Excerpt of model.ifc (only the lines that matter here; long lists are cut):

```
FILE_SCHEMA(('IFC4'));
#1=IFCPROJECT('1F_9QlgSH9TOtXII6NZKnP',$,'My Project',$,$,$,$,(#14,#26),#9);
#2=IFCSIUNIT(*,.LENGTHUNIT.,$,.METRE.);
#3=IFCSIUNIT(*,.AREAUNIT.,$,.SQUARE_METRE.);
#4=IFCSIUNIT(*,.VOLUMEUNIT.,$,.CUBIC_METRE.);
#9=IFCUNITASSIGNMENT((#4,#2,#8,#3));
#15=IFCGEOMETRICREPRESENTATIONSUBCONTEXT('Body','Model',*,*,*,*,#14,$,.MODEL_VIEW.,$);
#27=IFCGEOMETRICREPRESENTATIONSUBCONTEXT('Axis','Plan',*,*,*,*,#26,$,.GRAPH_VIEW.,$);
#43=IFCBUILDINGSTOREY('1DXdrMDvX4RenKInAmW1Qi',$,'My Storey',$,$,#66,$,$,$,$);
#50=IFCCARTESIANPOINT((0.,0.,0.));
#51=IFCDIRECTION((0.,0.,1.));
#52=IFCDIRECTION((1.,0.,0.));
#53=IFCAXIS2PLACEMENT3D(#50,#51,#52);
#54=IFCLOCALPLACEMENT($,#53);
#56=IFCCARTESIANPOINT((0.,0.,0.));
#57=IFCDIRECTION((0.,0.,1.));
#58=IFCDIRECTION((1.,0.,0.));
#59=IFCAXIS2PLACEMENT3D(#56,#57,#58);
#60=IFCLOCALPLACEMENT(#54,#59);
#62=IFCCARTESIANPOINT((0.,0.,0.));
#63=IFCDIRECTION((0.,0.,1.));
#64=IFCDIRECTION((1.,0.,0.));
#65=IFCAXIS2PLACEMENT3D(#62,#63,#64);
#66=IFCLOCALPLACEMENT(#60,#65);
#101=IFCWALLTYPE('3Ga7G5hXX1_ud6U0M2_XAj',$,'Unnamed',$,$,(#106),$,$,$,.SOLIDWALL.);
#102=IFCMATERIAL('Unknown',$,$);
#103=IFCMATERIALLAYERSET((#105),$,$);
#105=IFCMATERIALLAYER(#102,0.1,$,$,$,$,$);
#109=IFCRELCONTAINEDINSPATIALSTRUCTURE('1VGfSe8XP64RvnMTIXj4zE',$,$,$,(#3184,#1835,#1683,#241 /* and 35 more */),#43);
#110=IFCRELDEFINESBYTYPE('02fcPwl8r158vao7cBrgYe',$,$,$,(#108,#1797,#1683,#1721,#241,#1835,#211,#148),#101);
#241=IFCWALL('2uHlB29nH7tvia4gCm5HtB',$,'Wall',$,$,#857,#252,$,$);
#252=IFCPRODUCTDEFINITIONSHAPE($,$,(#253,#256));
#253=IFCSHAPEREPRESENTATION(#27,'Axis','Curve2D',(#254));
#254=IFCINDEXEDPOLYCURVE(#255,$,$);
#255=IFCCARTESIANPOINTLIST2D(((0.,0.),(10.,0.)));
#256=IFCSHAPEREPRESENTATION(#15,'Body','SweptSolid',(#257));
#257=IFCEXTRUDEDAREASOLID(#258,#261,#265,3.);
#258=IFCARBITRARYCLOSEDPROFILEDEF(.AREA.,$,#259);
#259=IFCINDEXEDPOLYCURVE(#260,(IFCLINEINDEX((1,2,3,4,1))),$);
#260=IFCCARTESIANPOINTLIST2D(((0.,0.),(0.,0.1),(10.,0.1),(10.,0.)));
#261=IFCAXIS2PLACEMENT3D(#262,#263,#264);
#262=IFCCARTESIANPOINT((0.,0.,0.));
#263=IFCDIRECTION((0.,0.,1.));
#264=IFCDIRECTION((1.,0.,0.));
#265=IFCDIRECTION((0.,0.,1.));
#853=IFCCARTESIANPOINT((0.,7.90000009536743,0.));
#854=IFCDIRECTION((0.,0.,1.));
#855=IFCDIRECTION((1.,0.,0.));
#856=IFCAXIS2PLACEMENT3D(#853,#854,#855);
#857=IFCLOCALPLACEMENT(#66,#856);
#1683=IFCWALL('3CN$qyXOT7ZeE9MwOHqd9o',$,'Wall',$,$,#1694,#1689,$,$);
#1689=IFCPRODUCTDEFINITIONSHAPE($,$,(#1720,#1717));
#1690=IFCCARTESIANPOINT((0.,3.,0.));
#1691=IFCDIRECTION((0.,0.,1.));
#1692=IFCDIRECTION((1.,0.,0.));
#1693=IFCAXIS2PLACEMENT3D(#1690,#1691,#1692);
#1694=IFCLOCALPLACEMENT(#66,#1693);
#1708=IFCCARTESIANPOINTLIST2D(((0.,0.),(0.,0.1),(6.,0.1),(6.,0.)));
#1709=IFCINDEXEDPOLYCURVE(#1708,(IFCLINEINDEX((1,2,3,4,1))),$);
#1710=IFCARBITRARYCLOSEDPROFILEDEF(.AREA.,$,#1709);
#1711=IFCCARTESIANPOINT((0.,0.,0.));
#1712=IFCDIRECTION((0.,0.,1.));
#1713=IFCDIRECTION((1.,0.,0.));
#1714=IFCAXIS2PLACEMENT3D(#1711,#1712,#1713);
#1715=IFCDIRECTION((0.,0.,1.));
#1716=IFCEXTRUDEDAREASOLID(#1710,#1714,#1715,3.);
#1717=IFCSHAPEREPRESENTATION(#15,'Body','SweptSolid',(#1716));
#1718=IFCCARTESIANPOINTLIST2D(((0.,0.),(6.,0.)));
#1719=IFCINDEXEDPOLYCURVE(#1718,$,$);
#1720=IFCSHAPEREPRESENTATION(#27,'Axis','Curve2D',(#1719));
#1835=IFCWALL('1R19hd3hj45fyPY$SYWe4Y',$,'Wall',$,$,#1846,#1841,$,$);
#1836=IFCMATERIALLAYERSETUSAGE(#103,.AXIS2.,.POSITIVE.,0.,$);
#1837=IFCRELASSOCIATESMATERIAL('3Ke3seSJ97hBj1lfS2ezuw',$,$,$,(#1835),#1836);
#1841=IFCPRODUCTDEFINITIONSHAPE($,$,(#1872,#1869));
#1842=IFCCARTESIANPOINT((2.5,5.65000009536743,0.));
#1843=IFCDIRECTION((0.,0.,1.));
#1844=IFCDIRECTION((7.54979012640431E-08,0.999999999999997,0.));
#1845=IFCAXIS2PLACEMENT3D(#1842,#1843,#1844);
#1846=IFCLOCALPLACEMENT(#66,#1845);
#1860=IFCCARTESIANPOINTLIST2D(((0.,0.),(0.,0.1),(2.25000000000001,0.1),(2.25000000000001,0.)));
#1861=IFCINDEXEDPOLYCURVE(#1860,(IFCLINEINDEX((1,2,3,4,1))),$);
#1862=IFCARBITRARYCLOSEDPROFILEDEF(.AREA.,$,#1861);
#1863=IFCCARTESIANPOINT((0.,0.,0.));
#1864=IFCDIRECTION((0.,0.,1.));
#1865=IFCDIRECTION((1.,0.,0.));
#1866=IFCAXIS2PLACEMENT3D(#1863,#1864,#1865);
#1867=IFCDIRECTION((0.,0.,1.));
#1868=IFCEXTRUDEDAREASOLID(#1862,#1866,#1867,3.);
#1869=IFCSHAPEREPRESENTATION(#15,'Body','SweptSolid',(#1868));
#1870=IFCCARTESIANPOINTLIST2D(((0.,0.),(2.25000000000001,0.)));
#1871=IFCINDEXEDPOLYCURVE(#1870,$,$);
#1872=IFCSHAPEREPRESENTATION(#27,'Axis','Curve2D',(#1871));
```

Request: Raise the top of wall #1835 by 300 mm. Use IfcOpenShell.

```python
import ifcopenshell
import ifcopenshell.geom
import ifcopenshell.util.representation
import ifcopenshell.util.shape

model = ifcopenshell.open("model.ifc")
settings = ifcopenshell.geom.settings()


def volume(element):
    """Net volume in cubic metres, openings subtracted."""
    shape = ifcopenshell.geom.create_shape(settings, element)
    return ifcopenshell.util.shape.get_volume(shape.geometry)


wall = model.by_id(1835)
before = volume(wall)

body = ifcopenshell.util.representation.get_representation(wall, "Model", "Body")
solid = body.Items[0]
old_height = solid.Depth
solid.Depth += 0.3
after = volume(wall)

print(f"height {old_height:g} -> {solid.Depth:g}, volume {before:.3f} -> {after:.3f} m3")

model.write("model_updated.ifc")
```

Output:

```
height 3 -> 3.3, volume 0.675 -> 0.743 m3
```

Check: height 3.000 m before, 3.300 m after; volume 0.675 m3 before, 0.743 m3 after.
